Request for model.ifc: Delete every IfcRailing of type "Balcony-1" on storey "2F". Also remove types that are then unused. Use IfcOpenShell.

First a look at what the model holds.

```python
import ifcopenshell
import ifcopenshell.util.element

model = ifcopenshell.open("model.ifc")
print(model.schema)
storey = next(s for s in model.by_type("IfcBuildingStorey") if s.Name == "2F")
railings = [e for e in ifcopenshell.util.element.get_decomposition(storey) if e.is_a("IfcRailing")]
seen = {}
for e in railings:
    element_type = ifcopenshell.util.element.get_type(e)
    name = element_type.Name if element_type not in (None, e) else None
    seen[name] = seen.get(name, 0) + 1
for name, count in sorted(seen.items(), key=str):
    print(count, "x", name)
```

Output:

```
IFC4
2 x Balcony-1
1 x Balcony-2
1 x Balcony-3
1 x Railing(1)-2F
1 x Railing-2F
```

```python
import ifcopenshell
import ifcopenshell.api.root
import ifcopenshell.util.element

model = ifcopenshell.open("model.ifc")

storey = next(s for s in model.by_type("IfcBuildingStorey") if s.Name == "2F")
railings = [e for e in ifcopenshell.util.element.get_decomposition(storey) if e.is_a("IfcRailing")]
targets = [e for e in railings if (t := ifcopenshell.util.element.get_type(e)) not in (None, e) and t.Name == "Balcony-1"]
types = {ifcopenshell.util.element.get_type(e) for e in targets} - {None, *targets}

for e in targets:
    ifcopenshell.api.root.remove_product(model, product=e)
print(len(targets), "removed")

unused = [t for t in types if not ifcopenshell.util.element.get_types(t)]
for t in unused:
    ifcopenshell.api.root.remove_product(model, product=t)
print(len(unused), "unused types removed")

model.write("model_v2.ifc")
```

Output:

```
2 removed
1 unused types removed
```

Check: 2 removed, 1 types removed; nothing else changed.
